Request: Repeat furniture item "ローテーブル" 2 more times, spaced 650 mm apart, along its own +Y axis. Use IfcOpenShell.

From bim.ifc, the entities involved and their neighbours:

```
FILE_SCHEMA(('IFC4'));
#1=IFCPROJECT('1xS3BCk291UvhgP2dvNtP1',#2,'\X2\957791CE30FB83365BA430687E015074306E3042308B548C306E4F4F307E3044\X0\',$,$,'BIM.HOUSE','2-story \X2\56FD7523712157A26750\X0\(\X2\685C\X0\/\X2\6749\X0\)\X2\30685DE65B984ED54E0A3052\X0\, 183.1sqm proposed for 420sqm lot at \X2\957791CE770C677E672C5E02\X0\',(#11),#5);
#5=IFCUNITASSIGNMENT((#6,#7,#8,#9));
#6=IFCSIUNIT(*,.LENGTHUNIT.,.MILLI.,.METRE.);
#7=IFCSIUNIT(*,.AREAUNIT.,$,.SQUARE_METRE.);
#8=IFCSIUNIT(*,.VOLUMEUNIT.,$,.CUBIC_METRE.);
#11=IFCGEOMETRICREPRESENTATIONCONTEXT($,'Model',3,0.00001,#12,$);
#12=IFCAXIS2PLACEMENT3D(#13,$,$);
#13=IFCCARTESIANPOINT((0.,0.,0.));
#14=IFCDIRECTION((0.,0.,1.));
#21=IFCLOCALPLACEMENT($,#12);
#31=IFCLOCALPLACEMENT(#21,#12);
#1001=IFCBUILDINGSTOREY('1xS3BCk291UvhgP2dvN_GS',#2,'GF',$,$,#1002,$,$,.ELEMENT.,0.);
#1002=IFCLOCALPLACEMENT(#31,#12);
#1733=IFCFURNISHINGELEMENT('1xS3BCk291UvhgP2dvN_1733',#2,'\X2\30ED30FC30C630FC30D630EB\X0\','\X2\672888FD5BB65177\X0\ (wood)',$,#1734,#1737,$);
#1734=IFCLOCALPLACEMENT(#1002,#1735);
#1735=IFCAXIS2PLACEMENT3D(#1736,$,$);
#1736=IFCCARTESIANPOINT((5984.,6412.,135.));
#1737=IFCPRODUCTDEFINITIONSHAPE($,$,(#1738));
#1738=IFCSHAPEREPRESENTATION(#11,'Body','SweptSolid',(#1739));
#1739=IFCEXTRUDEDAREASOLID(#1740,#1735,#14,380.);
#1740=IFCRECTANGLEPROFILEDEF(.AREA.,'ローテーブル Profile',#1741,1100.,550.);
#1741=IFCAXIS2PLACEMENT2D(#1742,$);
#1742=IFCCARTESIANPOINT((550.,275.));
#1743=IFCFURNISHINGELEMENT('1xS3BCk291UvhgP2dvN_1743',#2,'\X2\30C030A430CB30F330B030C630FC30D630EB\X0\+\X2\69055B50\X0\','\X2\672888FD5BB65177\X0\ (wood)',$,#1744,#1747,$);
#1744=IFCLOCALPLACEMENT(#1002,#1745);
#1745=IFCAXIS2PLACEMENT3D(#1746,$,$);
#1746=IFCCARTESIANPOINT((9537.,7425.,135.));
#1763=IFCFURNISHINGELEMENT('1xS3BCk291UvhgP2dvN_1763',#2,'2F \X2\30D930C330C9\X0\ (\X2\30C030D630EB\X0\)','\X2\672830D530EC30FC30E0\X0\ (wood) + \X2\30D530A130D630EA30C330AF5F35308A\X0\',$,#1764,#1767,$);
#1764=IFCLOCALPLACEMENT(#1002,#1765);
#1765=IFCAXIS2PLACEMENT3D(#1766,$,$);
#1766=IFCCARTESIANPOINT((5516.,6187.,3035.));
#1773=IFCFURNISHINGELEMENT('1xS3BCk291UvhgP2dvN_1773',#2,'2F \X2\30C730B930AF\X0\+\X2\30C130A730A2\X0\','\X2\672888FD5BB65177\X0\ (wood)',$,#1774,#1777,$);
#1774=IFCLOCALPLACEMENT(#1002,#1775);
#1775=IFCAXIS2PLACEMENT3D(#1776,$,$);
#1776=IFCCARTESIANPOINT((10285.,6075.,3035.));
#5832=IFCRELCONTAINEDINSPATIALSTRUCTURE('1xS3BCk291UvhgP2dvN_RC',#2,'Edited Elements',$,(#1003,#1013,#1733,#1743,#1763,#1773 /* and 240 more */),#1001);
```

```python
import ifcopenshell
import ifcopenshell.api.geometry
import ifcopenshell.api.root
import ifcopenshell.util.element
import ifcopenshell.util.placement

model = ifcopenshell.open("bim.ifc")


def reuse_history(source, copy):
    """copy_class also copies each property set's owner history, people and application; keep the originals."""
    for rel in copy.IsDefinedBy:
        if rel.is_a("IfcRelDefinesByProperties") and (history := rel.RelatingPropertyDefinition.OwnerHistory):
            rel.RelatingPropertyDefinition.OwnerHistory = source.OwnerHistory
            ifcopenshell.util.element.remove_deep2(model, history)


source = model.by_guid("1xS3BCk291UvhgP2dvN_1733")
base = ifcopenshell.util.placement.get_local_placement(source.ObjectPlacement)
step = base[:3, 1] * 650.0

for i in range(1, 3):
    copy = ifcopenshell.api.root.copy_class(model, product=source)
    copy.Representation = ifcopenshell.util.element.copy_deep(
        model, source.Representation, exclude=["IfcGeometricRepresentationContext", "IfcRepresentationMap"]
    )
    reuse_history(source, copy)
    matrix = base.copy()
    matrix[:3, 3] += i * step
    print("added at", matrix[:3, 3].round(3) + 0.0)
    ifcopenshell.api.geometry.edit_object_placement(model, product=copy, matrix=matrix, is_si=False)

model.write("bim-out.ifc")
```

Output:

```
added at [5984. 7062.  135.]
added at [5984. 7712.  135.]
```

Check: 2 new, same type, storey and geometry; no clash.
